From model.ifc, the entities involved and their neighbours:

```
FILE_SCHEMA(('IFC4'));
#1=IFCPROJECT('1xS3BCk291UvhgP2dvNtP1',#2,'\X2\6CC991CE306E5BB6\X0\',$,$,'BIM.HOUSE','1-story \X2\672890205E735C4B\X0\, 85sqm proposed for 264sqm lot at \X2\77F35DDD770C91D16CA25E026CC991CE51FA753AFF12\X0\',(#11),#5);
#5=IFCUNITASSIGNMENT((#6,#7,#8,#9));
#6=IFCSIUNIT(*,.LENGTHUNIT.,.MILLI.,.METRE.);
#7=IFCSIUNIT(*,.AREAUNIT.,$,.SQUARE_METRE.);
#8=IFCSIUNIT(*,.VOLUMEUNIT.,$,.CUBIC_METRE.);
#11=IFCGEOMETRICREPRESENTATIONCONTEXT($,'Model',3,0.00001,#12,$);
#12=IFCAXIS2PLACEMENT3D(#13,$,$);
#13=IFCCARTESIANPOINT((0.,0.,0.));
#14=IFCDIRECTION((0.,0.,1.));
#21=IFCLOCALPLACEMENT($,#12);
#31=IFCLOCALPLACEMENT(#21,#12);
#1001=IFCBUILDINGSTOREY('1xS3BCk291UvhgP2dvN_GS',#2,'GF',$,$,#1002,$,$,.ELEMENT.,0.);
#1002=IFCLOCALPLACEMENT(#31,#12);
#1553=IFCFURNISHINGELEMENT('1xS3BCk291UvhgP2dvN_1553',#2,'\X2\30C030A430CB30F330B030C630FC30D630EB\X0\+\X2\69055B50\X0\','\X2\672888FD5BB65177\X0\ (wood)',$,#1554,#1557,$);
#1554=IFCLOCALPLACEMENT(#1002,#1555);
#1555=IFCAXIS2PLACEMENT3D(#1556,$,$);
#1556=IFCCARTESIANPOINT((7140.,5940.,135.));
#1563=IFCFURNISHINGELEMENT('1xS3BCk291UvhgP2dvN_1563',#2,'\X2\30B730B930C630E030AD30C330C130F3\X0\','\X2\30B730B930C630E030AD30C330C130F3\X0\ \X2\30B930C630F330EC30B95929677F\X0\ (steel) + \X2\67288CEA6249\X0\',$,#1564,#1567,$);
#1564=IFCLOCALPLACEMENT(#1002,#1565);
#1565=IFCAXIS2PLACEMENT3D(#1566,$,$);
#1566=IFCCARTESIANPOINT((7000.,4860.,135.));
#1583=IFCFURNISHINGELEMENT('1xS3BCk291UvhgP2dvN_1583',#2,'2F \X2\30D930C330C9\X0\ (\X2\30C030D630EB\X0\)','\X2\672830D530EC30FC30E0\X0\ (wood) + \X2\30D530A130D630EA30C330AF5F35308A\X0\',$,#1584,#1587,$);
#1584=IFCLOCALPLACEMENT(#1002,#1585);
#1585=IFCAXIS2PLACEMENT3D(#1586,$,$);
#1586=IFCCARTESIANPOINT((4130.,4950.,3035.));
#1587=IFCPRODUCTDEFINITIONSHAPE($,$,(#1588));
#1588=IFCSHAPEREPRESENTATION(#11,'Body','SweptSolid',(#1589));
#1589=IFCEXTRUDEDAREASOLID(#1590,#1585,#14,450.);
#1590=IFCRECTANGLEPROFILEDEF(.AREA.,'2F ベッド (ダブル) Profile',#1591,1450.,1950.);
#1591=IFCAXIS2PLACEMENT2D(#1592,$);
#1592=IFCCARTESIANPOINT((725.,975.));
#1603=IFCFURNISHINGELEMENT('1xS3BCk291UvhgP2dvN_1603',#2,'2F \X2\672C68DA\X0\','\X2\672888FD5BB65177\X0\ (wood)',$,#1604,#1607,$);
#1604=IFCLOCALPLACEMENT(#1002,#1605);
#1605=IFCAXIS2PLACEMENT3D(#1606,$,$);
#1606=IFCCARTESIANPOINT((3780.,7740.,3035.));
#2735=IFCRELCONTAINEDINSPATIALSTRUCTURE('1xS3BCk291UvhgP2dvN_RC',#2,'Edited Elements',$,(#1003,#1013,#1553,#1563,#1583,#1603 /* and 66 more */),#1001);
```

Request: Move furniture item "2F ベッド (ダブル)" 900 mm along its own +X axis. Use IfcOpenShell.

```python
import ifcopenshell
import ifcopenshell.api.geometry
import ifcopenshell.util.placement
import ifcopenshell.util.unit

model = ifcopenshell.open("model.ifc")
unit_scale = ifcopenshell.util.unit.calculate_unit_scale(model)

item = model.by_guid("1xS3BCk291UvhgP2dvN_1583")
matrix = ifcopenshell.util.placement.get_local_placement(item.ObjectPlacement)
matrix[:3, 3] += matrix[:3, 0] * 0.9 / unit_scale
ifcopenshell.api.geometry.edit_object_placement(model, product=item, matrix=matrix, is_si=False)

print(ifcopenshell.util.placement.get_local_placement(item.ObjectPlacement).round(3) + 0.0)

model.write("model_v2.ifc")
```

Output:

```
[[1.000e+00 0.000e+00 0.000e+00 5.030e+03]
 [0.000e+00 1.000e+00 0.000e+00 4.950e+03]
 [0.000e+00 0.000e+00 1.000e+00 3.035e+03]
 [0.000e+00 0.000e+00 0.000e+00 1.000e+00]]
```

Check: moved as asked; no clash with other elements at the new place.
